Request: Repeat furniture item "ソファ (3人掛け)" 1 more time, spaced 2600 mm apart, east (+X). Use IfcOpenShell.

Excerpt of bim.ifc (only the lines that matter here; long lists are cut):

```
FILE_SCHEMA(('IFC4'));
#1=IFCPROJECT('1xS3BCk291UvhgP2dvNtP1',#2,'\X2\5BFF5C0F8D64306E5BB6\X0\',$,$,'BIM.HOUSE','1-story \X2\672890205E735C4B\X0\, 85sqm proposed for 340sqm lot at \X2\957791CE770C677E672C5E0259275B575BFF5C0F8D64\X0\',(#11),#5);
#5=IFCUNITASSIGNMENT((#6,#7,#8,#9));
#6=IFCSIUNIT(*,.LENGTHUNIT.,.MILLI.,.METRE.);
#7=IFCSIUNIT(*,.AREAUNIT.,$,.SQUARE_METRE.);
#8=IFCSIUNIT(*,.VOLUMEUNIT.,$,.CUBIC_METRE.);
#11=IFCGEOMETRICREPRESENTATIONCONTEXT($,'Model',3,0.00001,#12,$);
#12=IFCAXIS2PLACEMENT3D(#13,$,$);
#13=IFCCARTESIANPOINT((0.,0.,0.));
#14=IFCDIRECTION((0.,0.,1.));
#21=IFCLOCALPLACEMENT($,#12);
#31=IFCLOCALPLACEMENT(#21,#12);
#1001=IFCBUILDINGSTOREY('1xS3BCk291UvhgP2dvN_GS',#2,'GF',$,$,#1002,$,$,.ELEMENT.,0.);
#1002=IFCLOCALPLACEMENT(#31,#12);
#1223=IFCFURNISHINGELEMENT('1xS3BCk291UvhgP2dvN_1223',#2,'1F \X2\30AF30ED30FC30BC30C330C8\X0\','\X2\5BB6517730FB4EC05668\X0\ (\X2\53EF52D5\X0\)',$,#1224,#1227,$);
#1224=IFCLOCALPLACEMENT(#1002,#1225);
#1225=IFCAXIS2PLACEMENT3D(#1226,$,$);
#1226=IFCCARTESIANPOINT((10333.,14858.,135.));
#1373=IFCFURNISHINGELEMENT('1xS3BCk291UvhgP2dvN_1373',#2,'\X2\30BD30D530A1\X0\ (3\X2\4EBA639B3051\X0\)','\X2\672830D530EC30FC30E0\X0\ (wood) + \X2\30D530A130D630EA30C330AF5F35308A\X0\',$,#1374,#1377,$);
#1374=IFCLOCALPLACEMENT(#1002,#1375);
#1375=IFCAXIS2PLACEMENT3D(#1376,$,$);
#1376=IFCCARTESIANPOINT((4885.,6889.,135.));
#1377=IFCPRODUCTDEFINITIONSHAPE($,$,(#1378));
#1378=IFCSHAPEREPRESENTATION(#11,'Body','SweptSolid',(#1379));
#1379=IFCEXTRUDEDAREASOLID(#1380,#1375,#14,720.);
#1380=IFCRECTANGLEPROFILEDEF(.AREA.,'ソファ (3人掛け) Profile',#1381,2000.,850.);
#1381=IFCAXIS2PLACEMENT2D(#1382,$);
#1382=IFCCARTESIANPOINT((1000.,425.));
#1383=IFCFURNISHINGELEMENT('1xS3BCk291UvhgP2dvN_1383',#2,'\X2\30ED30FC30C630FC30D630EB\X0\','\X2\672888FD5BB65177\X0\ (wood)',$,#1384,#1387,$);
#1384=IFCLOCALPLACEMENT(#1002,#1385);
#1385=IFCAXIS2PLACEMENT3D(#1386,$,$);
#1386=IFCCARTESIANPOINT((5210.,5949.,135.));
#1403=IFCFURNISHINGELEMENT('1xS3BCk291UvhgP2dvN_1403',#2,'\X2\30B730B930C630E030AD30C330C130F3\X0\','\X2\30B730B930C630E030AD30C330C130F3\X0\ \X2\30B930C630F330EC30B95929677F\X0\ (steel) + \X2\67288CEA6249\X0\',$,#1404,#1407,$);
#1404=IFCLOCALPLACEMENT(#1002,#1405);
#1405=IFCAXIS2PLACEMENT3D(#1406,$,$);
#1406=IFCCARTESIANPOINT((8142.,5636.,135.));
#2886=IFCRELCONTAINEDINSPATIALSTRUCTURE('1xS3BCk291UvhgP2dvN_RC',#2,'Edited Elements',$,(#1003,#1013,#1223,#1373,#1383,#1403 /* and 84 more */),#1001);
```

```python
import numpy as np
import ifcopenshell
import ifcopenshell.api.geometry
import ifcopenshell.api.root
import ifcopenshell.util.element
import ifcopenshell.util.placement

model = ifcopenshell.open("bim.ifc")


def reuse_history(source, copy):
    """copy_class also copies each property set's owner history, people and application; keep the originals."""
    for rel in copy.IsDefinedBy:
        if rel.is_a("IfcRelDefinesByProperties") and (history := rel.RelatingPropertyDefinition.OwnerHistory):
            rel.RelatingPropertyDefinition.OwnerHistory = source.OwnerHistory
            ifcopenshell.util.element.remove_deep2(model, history)


source = model.by_guid("1xS3BCk291UvhgP2dvN_1373")
base = ifcopenshell.util.placement.get_local_placement(source.ObjectPlacement)
step = np.array([1.0, 0.0, 0.0]) * 2600.0

for i in range(1, 2):
    copy = ifcopenshell.api.root.copy_class(model, product=source)
    copy.Representation = ifcopenshell.util.element.copy_deep(
        model, source.Representation, exclude=["IfcGeometricRepresentationContext", "IfcRepresentationMap"]
    )
    reuse_history(source, copy)
    matrix = base.copy()
    matrix[:3, 3] += i * step
    print("added at", matrix[:3, 3].round(3) + 0.0)
    ifcopenshell.api.geometry.edit_object_placement(model, product=copy, matrix=matrix, is_si=False)

model.write("bim_rev.ifc")
```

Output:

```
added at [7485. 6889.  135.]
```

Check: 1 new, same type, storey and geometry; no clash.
